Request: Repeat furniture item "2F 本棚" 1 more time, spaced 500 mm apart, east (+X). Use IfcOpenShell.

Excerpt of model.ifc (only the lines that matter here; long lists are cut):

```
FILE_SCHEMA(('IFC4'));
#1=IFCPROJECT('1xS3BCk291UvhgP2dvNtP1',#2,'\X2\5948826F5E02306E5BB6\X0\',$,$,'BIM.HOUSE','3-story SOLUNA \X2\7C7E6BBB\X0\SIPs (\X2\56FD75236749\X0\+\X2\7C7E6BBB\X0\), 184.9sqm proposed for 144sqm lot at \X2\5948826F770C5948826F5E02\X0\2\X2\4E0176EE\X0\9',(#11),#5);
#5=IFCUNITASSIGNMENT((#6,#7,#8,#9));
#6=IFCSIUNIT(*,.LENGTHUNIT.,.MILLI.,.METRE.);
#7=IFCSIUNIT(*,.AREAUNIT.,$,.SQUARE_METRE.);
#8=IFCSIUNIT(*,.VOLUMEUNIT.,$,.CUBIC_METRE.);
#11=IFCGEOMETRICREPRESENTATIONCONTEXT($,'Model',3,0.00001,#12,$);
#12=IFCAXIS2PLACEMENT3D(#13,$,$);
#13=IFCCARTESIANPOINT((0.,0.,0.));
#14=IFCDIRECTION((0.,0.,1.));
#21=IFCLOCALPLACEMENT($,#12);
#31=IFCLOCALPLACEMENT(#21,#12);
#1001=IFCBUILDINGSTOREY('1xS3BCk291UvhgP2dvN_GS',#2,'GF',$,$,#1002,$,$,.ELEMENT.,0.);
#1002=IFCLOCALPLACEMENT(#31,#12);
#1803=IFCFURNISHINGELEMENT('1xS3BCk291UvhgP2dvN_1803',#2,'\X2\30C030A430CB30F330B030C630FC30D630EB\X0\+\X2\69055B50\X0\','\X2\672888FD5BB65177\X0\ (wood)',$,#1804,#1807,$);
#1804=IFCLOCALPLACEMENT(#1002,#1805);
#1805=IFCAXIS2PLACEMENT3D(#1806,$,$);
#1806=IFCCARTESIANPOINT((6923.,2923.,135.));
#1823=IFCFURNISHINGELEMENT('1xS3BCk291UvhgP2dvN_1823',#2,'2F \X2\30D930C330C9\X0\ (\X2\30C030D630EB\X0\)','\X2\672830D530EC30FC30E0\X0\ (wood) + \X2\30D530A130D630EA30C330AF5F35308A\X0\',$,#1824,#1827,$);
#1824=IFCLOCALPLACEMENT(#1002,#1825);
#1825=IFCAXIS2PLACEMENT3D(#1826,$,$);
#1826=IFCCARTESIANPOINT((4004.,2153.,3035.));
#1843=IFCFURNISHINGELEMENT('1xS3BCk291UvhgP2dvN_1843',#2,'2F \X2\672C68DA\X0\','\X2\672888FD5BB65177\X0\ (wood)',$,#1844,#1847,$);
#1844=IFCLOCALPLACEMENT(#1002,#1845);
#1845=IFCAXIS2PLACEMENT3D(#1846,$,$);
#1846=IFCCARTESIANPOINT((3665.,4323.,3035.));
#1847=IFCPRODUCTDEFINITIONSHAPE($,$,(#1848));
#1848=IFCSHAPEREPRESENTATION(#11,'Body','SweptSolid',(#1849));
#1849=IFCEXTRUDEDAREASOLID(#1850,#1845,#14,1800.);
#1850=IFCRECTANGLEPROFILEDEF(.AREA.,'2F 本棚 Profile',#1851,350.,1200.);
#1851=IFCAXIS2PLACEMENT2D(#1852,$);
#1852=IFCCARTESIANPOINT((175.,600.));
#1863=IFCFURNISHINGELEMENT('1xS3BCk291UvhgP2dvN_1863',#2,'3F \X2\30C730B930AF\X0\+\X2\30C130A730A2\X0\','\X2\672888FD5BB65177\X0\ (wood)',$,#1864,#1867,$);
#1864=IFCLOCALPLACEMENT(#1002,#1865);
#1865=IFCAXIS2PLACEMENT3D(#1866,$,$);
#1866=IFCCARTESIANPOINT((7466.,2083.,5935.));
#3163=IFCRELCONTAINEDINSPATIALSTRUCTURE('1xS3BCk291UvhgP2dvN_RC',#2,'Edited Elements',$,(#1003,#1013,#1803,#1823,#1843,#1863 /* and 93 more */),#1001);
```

```python
import numpy as np
import ifcopenshell
import ifcopenshell.api.geometry
import ifcopenshell.api.root
import ifcopenshell.util.element
import ifcopenshell.util.placement
import ifcopenshell.util.unit

model = ifcopenshell.open("model.ifc")
unit_scale = ifcopenshell.util.unit.calculate_unit_scale(model)


def reuse_history(source, copy):
    """copy_class also copies each property set's owner history, people and application; keep the originals."""
    for rel in copy.IsDefinedBy:
        if rel.is_a("IfcRelDefinesByProperties") and (history := rel.RelatingPropertyDefinition.OwnerHistory):
            rel.RelatingPropertyDefinition.OwnerHistory = source.OwnerHistory
            ifcopenshell.util.element.remove_deep2(model, history)


source = model.by_guid("1xS3BCk291UvhgP2dvN_1843")
base = ifcopenshell.util.placement.get_local_placement(source.ObjectPlacement)
step = np.array([1.0, 0.0, 0.0]) * 0.5 / unit_scale

for i in range(1, 2):
    copy = ifcopenshell.api.root.copy_class(model, product=source)
    copy.Representation = ifcopenshell.util.element.copy_deep(
        model, source.Representation, exclude=["IfcGeometricRepresentationContext", "IfcRepresentationMap"]
    )
    reuse_history(source, copy)
    matrix = base.copy()
    matrix[:3, 3] += i * step
    print("added at", matrix[:3, 3].round(3) + 0.0)
    ifcopenshell.api.geometry.edit_object_placement(model, product=copy, matrix=matrix, is_si=False)

model.write("model_updated.ifc")
```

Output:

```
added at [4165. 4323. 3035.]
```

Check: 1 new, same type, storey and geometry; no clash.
